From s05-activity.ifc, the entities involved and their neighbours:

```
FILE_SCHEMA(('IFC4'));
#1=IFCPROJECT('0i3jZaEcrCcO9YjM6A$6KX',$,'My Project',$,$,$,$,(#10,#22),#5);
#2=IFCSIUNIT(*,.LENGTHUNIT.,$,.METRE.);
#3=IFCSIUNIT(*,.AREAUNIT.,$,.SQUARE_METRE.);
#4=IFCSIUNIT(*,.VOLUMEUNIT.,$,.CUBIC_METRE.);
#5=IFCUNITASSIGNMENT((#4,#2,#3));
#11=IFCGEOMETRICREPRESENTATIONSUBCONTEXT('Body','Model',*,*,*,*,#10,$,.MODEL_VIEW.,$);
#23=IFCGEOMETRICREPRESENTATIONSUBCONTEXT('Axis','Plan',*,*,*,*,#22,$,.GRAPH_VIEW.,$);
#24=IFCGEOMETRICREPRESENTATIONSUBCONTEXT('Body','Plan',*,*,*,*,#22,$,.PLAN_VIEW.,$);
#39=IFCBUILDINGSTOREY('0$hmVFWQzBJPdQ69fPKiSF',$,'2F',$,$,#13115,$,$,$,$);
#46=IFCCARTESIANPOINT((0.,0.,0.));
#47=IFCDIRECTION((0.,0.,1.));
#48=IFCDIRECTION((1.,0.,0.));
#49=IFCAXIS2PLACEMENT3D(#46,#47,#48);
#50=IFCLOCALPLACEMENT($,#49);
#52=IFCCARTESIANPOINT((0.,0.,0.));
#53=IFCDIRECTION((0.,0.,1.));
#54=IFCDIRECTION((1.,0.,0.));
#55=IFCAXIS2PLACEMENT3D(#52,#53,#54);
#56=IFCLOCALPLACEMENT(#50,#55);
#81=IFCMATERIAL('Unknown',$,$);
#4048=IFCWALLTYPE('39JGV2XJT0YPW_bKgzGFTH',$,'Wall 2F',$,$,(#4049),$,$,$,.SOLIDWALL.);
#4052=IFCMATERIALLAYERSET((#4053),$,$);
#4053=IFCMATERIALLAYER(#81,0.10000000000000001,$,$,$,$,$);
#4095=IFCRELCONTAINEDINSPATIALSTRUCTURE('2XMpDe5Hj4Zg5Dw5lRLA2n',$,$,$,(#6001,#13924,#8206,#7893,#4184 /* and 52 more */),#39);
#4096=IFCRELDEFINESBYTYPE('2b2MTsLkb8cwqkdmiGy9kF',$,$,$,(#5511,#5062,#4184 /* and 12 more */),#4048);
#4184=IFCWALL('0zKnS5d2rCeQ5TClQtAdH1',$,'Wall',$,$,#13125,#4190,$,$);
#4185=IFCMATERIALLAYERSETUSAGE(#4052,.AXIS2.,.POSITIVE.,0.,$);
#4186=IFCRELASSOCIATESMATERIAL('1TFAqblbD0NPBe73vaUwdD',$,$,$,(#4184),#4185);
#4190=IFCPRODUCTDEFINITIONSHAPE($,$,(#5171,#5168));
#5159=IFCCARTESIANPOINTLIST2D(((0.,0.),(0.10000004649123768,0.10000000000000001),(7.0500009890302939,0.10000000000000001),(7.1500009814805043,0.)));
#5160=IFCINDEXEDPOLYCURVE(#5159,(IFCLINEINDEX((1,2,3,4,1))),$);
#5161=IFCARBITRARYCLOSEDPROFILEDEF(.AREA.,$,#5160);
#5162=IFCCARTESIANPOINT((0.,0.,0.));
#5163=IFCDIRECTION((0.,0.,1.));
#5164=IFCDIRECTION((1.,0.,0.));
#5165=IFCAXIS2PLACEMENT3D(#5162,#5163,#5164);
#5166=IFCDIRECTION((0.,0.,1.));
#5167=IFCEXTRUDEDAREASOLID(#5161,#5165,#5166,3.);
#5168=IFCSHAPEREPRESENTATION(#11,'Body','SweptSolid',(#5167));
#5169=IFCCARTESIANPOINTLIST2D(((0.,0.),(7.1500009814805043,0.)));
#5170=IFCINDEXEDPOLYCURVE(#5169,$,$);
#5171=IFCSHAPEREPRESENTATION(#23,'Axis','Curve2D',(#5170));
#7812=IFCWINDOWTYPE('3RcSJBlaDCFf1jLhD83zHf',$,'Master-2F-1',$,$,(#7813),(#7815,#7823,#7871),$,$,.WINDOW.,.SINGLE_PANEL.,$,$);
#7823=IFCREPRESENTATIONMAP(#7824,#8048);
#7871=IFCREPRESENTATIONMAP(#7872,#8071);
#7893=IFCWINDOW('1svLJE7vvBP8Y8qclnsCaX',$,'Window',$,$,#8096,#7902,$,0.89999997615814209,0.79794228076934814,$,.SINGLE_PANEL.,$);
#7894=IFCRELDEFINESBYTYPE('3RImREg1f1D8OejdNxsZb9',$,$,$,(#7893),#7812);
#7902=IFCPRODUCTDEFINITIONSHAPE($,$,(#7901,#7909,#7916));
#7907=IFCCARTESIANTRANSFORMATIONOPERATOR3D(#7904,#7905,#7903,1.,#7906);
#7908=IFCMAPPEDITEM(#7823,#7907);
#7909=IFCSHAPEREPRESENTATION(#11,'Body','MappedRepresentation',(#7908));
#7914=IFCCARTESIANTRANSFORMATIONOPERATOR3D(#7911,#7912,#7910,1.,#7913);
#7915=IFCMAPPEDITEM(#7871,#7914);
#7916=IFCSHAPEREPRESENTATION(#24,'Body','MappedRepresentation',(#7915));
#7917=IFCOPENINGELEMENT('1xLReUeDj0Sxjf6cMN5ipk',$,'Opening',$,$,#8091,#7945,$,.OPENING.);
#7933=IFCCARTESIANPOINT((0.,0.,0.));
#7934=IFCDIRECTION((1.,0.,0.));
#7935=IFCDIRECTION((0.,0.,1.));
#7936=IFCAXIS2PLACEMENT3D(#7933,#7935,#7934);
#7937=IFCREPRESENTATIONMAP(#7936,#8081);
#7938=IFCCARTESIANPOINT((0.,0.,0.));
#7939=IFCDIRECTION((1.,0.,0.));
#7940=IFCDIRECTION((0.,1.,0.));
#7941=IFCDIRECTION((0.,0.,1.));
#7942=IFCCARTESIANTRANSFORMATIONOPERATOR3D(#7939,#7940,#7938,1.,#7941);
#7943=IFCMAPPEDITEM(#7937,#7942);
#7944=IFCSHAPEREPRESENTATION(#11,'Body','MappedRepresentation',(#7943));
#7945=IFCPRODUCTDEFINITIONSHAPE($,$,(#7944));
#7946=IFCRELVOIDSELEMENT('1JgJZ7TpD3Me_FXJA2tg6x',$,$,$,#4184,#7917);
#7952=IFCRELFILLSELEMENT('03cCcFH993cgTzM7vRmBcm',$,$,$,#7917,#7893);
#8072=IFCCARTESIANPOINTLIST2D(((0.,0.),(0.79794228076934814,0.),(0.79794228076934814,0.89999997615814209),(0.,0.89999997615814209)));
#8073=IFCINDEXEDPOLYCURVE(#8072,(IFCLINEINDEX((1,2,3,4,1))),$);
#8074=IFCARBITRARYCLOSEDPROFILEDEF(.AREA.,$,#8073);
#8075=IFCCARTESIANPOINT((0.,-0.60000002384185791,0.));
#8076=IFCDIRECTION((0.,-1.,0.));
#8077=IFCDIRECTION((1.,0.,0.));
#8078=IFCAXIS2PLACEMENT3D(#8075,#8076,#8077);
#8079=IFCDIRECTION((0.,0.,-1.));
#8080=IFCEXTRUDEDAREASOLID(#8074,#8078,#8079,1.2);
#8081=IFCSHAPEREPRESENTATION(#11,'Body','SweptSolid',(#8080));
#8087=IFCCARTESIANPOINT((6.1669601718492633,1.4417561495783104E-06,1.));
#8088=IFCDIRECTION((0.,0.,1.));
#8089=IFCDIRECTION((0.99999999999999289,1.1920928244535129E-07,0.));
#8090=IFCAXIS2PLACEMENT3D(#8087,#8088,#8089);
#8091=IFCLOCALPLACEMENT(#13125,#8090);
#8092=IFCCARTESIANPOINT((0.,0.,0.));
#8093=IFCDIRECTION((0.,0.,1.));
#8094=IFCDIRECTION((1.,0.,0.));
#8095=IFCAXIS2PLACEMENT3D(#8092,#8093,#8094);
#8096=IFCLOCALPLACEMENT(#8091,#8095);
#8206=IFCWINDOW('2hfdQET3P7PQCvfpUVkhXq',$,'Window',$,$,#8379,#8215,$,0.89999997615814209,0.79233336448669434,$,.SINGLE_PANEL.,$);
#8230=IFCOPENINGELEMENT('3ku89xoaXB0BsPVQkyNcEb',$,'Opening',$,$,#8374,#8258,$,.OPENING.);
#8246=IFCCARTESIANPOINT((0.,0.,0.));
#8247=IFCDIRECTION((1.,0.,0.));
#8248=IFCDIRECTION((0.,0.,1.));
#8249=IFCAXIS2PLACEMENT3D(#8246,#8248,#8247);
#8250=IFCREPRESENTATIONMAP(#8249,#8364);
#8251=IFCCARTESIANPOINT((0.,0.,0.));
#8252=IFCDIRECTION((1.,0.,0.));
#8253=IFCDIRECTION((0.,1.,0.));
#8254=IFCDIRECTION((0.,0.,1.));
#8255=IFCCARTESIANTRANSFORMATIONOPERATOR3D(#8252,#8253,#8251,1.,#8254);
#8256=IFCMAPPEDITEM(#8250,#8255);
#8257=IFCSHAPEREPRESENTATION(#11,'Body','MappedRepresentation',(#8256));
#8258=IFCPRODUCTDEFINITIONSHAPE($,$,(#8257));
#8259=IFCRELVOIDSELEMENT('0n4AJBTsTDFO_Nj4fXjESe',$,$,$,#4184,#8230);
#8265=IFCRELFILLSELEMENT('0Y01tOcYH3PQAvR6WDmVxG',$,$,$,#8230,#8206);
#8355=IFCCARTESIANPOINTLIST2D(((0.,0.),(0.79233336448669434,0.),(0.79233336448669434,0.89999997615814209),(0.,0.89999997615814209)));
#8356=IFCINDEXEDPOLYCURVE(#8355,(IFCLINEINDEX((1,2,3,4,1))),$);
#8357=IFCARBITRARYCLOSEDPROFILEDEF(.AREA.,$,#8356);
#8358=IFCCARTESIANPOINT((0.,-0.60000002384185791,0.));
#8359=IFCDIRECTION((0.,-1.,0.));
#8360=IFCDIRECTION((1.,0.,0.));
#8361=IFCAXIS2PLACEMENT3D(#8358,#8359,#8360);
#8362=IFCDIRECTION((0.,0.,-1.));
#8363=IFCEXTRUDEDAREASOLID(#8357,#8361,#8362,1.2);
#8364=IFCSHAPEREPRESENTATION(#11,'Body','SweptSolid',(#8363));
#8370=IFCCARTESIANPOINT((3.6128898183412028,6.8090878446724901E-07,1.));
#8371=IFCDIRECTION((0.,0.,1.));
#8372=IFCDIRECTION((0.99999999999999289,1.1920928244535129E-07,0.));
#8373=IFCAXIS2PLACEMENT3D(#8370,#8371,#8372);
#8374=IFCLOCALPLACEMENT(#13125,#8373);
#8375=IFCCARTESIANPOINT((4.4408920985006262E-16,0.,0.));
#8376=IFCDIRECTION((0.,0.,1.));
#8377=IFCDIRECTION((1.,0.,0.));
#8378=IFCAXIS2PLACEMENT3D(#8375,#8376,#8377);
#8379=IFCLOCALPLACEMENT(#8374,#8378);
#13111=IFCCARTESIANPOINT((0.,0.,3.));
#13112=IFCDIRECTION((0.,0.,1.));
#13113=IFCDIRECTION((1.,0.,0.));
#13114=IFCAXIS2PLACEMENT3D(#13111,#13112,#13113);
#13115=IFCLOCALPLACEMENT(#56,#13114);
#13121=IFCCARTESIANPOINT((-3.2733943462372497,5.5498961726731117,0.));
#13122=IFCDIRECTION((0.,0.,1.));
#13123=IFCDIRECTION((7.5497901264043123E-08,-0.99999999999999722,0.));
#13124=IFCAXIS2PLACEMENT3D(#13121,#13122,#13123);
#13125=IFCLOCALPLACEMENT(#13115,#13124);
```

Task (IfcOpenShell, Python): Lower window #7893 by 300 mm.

```python
import numpy as np
import ifcopenshell
import ifcopenshell.api.geometry
import ifcopenshell.util.placement
import ifcopenshell.util.unit

model = ifcopenshell.open("s05-activity.ifc")
unit_scale = ifcopenshell.util.unit.calculate_unit_scale(model)

window = model.by_guid("1svLJE7vvBP8Y8qclnsCaX")
opening = window.FillsVoids[0].RelatingOpeningElement
dz = -0.3 / unit_scale

shift = np.array([0.0, 0.0, dz])
# The window is placed relative to its opening, so it follows when the opening moves.
matrix = ifcopenshell.util.placement.get_local_placement(opening.ObjectPlacement)
matrix[:3, 3] += shift
ifcopenshell.api.geometry.edit_object_placement(
    model, product=opening, matrix=matrix, is_si=False, should_transform_children=True
)

print(f"moved by {dz * unit_scale:+.3f} m")

model.write("s05-activity_v2.ifc")
```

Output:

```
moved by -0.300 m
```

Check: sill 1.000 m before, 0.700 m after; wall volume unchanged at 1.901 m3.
